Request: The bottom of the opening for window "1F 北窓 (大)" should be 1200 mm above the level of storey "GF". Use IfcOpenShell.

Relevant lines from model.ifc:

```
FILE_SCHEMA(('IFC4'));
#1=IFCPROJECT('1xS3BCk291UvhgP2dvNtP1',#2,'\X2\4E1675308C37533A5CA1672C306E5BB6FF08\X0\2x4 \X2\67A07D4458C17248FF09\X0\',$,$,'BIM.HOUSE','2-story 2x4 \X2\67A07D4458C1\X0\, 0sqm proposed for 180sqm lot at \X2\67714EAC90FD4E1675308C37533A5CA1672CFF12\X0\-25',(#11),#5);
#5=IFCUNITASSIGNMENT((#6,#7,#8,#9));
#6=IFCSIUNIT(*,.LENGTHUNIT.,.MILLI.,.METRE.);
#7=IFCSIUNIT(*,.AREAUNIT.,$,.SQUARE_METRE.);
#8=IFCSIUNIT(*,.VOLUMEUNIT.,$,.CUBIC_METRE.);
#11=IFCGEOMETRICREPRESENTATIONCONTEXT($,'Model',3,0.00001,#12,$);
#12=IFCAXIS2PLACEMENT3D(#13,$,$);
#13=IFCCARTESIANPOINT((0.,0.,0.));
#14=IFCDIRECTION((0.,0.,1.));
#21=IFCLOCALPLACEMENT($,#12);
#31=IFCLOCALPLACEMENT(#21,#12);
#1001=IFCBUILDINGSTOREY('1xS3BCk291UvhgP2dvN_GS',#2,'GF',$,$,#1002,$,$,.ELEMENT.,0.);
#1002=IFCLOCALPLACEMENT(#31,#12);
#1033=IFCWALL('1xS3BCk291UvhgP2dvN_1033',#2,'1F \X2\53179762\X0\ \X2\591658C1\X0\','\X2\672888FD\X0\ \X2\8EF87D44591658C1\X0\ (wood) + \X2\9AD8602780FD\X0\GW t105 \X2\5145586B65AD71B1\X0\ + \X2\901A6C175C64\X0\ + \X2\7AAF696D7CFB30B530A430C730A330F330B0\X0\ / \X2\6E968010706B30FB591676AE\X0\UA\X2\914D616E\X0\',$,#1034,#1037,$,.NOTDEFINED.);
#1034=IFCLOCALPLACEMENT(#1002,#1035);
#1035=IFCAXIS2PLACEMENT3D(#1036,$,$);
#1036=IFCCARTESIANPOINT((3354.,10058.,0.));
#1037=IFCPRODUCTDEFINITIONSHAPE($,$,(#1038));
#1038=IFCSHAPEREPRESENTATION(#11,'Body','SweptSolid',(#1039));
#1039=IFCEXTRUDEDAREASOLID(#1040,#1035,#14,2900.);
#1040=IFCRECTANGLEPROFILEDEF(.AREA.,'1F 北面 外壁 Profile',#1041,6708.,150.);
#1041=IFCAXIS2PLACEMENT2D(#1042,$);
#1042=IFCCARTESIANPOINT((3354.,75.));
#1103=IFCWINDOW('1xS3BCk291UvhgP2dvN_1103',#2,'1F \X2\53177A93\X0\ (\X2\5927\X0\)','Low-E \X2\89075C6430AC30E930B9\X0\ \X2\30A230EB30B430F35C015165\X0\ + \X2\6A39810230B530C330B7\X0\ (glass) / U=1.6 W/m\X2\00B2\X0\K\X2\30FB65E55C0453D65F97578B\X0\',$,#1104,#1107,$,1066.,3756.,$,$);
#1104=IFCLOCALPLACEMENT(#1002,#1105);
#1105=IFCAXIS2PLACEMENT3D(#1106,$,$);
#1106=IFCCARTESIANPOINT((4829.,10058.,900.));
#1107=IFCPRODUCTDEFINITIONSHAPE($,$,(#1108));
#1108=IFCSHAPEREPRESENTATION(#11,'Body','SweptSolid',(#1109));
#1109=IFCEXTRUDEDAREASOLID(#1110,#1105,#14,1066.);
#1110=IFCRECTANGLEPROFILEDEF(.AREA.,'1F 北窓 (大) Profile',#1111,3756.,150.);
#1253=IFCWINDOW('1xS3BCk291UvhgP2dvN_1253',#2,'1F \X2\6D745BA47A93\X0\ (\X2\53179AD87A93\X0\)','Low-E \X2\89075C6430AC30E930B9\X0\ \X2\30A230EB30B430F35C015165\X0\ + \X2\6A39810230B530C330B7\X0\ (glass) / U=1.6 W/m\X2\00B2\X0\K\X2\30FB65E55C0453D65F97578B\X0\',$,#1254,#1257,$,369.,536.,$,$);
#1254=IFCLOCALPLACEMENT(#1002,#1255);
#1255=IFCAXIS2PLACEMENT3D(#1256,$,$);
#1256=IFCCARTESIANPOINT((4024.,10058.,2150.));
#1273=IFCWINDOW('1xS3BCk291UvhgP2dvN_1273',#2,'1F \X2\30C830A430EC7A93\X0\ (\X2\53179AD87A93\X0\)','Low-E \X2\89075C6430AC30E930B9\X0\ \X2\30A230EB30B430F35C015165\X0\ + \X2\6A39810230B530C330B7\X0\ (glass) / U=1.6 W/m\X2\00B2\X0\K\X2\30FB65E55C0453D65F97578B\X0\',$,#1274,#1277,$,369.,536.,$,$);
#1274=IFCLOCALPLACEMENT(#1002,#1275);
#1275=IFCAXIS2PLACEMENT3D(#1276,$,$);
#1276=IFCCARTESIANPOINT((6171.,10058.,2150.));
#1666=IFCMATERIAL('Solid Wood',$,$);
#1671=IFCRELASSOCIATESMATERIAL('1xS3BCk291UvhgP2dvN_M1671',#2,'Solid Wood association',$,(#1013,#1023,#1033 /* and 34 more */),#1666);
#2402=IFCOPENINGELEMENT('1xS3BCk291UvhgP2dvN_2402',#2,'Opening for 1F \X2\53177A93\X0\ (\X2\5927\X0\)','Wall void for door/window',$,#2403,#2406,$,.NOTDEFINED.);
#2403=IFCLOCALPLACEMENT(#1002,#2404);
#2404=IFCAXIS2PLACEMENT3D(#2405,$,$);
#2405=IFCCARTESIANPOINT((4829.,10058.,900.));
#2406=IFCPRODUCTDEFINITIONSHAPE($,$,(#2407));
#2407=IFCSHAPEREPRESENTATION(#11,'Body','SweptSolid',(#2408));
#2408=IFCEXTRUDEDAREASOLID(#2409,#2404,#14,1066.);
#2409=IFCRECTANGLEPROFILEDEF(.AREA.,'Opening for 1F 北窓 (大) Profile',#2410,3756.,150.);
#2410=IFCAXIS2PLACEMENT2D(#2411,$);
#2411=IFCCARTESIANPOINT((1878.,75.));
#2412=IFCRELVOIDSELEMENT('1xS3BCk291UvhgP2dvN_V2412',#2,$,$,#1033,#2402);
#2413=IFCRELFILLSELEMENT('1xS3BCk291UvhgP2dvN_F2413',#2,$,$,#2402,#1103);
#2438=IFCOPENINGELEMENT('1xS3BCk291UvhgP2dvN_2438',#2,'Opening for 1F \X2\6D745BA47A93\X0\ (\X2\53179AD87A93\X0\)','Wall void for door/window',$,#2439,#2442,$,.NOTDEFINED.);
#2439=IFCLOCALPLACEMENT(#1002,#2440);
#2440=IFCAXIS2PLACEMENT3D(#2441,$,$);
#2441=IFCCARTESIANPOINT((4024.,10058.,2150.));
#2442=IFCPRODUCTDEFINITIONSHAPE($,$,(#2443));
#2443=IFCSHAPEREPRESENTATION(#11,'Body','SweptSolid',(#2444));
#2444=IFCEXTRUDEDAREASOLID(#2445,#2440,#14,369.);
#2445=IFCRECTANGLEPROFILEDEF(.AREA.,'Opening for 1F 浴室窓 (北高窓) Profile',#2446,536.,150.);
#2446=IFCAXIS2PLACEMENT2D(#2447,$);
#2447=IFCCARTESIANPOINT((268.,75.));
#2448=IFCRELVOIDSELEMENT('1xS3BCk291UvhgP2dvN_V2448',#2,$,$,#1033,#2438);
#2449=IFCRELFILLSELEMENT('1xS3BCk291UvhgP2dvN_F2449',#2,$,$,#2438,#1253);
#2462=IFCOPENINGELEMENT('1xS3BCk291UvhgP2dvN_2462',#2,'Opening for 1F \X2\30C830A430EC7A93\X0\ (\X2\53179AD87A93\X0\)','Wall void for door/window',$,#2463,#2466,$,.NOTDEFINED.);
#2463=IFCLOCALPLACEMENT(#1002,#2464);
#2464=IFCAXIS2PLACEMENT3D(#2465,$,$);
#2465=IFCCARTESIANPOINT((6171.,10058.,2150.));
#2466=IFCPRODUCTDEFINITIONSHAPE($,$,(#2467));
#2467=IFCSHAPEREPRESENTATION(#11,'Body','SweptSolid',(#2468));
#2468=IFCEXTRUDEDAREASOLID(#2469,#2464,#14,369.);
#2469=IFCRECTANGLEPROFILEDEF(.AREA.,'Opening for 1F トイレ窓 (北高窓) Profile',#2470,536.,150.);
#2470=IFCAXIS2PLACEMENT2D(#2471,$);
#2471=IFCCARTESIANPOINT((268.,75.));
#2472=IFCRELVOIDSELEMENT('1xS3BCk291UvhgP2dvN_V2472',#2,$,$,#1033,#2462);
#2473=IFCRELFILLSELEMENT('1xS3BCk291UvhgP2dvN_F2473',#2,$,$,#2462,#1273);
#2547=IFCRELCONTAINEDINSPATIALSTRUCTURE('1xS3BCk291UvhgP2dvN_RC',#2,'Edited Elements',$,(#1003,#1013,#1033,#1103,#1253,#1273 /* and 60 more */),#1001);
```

```python
import numpy as np
import ifcopenshell
import ifcopenshell.api.geometry
import ifcopenshell.geom
import ifcopenshell.util.element
import ifcopenshell.util.placement
import ifcopenshell.util.shape
import ifcopenshell.util.unit

model = ifcopenshell.open("model.ifc")
unit_scale = ifcopenshell.util.unit.calculate_unit_scale(model)

window = model.by_id(1103)
opening = window.FillsVoids[0].RelatingOpeningElement
storey = ifcopenshell.util.element.get_container(window, ifc_class="IfcBuildingStorey")
level = ifcopenshell.util.placement.get_local_placement(storey.ObjectPlacement)[2, 3]

# The opening's origin need not be at the sill, so measure its lowest point.
shape = ifcopenshell.geom.create_shape(ifcopenshell.geom.settings(), opening)
bottom = ifcopenshell.util.shape.get_shape_bottom_elevation(shape, shape.geometry) / unit_scale
dz = level + 1200.0 - bottom

shift = np.array([0.0, 0.0, dz])
# The window is not placed relative to its opening, so move both.
for product in (opening, window):
    matrix = ifcopenshell.util.placement.get_local_placement(product.ObjectPlacement)
    matrix[:3, 3] += shift
    ifcopenshell.api.geometry.edit_object_placement(model, product=product, matrix=matrix, is_si=False)

print(f"moved by {dz * unit_scale:+.3f} m")

model.write("model_updated.ifc")
```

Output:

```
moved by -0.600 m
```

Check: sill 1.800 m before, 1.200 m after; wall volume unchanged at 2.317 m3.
